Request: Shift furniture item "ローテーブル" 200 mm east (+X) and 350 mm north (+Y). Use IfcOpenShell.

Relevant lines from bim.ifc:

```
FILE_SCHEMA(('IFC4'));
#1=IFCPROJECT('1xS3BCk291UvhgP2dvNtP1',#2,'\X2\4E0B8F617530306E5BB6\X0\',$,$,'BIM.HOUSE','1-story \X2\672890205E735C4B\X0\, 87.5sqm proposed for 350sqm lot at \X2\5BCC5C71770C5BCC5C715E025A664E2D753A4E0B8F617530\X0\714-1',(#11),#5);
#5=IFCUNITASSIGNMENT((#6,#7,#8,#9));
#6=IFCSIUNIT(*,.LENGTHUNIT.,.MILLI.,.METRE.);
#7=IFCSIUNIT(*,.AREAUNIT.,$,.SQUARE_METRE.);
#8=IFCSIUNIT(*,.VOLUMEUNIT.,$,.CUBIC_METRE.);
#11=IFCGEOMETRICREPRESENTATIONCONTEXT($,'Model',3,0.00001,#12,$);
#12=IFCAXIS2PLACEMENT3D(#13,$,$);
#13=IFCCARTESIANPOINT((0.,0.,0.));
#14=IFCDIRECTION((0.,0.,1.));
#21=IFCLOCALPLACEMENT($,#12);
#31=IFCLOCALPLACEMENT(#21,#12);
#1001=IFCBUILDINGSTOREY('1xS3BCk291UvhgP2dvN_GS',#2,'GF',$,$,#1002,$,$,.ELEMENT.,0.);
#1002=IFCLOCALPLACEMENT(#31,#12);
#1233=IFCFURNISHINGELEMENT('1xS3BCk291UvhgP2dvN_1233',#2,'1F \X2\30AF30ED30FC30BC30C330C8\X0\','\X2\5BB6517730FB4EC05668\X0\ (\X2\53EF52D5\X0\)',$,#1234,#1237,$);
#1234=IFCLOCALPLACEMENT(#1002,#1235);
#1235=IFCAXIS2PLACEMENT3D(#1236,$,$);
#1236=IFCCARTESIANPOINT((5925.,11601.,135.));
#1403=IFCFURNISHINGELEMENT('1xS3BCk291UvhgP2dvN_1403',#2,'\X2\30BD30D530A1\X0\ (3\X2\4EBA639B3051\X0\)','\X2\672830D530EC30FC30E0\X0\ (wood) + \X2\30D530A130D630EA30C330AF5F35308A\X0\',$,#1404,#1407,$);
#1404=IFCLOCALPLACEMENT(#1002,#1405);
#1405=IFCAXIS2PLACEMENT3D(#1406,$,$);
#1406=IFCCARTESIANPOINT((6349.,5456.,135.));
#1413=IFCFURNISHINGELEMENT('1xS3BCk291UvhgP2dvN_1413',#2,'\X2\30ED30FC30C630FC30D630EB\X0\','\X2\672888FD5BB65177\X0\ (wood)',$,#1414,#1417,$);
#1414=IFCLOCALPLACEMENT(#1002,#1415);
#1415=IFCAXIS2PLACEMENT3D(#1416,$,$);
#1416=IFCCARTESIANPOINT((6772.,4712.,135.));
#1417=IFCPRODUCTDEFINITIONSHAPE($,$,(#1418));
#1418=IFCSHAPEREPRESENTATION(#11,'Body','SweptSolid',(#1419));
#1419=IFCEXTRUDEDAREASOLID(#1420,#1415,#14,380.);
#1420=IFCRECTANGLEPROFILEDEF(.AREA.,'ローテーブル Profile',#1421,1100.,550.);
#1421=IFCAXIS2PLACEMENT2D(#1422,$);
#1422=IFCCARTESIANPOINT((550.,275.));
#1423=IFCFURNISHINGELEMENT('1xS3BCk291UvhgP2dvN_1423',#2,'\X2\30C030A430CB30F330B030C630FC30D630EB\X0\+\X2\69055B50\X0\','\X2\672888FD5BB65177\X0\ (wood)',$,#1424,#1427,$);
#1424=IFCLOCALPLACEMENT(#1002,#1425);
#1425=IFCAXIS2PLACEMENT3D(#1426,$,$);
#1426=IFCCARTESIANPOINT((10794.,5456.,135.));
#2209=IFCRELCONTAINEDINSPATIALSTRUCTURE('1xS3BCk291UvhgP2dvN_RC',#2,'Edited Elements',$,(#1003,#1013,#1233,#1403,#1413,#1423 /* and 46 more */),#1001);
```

```python
import ifcopenshell
import ifcopenshell.api.geometry
import ifcopenshell.util.placement
import ifcopenshell.util.unit

model = ifcopenshell.open("bim.ifc")
unit_scale = ifcopenshell.util.unit.calculate_unit_scale(model)

item = model.by_guid("1xS3BCk291UvhgP2dvN_1413")
matrix = ifcopenshell.util.placement.get_local_placement(item.ObjectPlacement)
matrix[0, 3] += 0.2 / unit_scale
matrix[1, 3] += 0.35 / unit_scale
ifcopenshell.api.geometry.edit_object_placement(model, product=item, matrix=matrix, is_si=False)

print(ifcopenshell.util.placement.get_local_placement(item.ObjectPlacement).round(3) + 0.0)

model.write("bim_v2.ifc")
```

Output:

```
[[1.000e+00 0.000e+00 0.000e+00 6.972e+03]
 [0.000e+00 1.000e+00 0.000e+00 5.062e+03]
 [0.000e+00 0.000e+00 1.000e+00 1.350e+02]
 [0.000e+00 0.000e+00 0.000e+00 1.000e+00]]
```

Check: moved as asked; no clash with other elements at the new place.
